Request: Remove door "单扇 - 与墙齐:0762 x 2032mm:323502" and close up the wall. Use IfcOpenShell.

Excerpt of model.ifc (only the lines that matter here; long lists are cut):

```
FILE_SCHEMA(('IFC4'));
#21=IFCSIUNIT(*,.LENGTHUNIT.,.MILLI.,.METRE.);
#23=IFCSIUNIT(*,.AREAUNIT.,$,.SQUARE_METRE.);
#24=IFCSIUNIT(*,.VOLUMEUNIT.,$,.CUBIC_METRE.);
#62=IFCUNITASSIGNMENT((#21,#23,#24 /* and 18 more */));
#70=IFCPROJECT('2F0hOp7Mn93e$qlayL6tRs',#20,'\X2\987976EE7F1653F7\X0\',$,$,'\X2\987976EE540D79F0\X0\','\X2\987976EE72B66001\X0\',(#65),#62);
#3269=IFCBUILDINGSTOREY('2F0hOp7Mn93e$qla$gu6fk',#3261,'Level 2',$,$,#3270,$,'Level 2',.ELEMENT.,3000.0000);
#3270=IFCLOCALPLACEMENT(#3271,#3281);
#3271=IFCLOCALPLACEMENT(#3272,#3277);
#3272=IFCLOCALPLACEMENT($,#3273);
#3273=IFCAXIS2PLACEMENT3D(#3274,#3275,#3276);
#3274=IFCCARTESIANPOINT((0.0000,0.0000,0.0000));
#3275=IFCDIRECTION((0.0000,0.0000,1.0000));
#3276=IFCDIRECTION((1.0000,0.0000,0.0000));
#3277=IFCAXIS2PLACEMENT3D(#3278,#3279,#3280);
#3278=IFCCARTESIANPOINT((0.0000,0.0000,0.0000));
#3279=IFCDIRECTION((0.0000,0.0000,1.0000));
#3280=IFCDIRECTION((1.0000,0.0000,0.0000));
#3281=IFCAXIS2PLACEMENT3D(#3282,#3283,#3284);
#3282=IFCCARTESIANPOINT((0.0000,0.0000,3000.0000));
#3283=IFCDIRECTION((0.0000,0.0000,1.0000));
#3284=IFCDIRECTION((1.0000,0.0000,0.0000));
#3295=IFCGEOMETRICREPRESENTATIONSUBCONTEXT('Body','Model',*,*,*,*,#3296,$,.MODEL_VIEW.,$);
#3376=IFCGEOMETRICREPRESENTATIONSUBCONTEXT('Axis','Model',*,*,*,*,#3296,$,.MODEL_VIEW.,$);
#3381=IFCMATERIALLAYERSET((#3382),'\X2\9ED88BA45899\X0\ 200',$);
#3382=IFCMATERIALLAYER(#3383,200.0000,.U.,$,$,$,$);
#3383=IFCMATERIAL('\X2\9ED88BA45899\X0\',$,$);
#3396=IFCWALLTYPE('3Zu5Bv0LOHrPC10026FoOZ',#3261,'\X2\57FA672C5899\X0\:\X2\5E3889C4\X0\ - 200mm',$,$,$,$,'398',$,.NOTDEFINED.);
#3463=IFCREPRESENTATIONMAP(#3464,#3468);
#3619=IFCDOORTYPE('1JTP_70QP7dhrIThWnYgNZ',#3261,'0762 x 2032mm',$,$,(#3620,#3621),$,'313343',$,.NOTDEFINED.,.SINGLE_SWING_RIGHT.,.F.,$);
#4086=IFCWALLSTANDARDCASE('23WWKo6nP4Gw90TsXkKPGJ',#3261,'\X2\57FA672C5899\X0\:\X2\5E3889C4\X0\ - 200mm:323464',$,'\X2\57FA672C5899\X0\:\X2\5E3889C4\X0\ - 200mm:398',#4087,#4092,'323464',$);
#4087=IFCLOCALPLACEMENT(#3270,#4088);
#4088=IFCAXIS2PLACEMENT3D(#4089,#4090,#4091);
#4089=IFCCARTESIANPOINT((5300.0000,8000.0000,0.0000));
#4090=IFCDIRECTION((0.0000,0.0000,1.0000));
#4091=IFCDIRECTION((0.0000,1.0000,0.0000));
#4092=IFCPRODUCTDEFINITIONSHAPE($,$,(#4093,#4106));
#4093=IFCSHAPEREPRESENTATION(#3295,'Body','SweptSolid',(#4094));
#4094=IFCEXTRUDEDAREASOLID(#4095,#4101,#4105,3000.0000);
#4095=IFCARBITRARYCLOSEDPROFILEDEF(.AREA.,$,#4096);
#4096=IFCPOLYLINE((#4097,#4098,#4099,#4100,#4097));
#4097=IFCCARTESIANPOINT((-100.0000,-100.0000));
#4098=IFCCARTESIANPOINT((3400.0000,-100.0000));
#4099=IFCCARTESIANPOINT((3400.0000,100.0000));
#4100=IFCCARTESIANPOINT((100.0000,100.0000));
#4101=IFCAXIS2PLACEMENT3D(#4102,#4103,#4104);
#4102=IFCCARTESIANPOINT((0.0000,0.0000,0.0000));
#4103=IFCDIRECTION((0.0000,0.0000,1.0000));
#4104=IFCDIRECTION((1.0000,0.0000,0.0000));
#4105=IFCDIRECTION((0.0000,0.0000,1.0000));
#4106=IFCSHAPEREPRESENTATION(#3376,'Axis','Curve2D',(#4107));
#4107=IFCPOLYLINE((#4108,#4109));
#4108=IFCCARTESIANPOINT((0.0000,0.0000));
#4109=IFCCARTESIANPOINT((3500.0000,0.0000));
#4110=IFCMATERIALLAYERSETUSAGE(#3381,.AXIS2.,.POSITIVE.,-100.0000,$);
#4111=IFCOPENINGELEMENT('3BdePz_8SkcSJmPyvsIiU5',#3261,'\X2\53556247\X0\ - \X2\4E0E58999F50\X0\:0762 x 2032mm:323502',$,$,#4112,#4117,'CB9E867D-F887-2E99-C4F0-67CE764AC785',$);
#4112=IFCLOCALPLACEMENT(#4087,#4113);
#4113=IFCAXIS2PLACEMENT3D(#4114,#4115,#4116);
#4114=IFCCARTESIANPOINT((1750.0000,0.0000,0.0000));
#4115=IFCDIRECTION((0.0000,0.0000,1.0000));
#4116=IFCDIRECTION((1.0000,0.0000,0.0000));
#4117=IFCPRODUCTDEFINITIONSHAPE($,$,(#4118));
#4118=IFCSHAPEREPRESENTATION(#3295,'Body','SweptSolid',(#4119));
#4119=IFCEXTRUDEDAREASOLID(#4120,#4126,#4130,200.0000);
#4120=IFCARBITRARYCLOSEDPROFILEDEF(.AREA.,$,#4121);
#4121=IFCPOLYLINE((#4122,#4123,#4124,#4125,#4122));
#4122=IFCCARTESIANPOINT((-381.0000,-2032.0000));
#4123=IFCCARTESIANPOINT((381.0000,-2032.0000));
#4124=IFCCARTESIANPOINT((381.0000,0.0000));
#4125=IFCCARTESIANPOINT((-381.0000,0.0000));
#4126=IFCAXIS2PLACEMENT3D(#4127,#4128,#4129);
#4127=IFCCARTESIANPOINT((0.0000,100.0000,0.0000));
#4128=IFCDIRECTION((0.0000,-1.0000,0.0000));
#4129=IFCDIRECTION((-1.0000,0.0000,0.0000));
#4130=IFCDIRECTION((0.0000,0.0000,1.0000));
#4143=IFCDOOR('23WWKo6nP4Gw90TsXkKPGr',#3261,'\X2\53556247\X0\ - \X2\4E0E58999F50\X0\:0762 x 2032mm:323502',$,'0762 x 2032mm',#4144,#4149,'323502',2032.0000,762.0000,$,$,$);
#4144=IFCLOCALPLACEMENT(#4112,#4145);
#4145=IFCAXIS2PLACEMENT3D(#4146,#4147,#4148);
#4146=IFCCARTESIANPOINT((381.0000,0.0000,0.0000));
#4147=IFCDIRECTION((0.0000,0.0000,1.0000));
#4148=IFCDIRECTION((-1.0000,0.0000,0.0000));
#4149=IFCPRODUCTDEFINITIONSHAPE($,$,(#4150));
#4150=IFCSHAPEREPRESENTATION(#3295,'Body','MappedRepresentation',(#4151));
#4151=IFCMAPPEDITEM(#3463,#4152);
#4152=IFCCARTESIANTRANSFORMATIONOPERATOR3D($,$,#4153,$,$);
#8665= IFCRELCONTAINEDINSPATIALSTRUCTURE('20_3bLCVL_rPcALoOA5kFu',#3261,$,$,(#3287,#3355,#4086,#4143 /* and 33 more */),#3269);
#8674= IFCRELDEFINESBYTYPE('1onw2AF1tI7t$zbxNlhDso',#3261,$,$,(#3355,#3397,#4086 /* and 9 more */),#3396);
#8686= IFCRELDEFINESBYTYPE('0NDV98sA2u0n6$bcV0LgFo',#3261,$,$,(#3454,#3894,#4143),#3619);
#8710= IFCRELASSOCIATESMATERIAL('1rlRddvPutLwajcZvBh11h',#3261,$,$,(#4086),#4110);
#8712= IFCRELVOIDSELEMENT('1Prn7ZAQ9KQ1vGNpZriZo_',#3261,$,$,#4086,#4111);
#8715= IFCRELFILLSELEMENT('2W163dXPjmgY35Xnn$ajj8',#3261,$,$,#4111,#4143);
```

```python
import ifcopenshell
import ifcopenshell.api.feature
import ifcopenshell.api.root
import ifcopenshell.geom
import ifcopenshell.util.shape

model = ifcopenshell.open("model.ifc")
settings = ifcopenshell.geom.settings()


def volume(element):
    """Net volume in cubic metres, openings subtracted."""
    shape = ifcopenshell.geom.create_shape(settings, element)
    return ifcopenshell.util.shape.get_volume(shape.geometry)


door = model.by_guid("23WWKo6nP4Gw90TsXkKPGr")
opening = door.FillsVoids[0].RelatingOpeningElement
wall = opening.VoidsElements[0].RelatingBuildingElement
before = volume(wall)

ifcopenshell.api.root.remove_product(model, product=door)
ifcopenshell.api.feature.remove_feature(model, feature=opening)

after = volume(wall)

print(f"wall volume {before:.3f} -> {after:.3f} m3")

model.write("model-out.ifc")
```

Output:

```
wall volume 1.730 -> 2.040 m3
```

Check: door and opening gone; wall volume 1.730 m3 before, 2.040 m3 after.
